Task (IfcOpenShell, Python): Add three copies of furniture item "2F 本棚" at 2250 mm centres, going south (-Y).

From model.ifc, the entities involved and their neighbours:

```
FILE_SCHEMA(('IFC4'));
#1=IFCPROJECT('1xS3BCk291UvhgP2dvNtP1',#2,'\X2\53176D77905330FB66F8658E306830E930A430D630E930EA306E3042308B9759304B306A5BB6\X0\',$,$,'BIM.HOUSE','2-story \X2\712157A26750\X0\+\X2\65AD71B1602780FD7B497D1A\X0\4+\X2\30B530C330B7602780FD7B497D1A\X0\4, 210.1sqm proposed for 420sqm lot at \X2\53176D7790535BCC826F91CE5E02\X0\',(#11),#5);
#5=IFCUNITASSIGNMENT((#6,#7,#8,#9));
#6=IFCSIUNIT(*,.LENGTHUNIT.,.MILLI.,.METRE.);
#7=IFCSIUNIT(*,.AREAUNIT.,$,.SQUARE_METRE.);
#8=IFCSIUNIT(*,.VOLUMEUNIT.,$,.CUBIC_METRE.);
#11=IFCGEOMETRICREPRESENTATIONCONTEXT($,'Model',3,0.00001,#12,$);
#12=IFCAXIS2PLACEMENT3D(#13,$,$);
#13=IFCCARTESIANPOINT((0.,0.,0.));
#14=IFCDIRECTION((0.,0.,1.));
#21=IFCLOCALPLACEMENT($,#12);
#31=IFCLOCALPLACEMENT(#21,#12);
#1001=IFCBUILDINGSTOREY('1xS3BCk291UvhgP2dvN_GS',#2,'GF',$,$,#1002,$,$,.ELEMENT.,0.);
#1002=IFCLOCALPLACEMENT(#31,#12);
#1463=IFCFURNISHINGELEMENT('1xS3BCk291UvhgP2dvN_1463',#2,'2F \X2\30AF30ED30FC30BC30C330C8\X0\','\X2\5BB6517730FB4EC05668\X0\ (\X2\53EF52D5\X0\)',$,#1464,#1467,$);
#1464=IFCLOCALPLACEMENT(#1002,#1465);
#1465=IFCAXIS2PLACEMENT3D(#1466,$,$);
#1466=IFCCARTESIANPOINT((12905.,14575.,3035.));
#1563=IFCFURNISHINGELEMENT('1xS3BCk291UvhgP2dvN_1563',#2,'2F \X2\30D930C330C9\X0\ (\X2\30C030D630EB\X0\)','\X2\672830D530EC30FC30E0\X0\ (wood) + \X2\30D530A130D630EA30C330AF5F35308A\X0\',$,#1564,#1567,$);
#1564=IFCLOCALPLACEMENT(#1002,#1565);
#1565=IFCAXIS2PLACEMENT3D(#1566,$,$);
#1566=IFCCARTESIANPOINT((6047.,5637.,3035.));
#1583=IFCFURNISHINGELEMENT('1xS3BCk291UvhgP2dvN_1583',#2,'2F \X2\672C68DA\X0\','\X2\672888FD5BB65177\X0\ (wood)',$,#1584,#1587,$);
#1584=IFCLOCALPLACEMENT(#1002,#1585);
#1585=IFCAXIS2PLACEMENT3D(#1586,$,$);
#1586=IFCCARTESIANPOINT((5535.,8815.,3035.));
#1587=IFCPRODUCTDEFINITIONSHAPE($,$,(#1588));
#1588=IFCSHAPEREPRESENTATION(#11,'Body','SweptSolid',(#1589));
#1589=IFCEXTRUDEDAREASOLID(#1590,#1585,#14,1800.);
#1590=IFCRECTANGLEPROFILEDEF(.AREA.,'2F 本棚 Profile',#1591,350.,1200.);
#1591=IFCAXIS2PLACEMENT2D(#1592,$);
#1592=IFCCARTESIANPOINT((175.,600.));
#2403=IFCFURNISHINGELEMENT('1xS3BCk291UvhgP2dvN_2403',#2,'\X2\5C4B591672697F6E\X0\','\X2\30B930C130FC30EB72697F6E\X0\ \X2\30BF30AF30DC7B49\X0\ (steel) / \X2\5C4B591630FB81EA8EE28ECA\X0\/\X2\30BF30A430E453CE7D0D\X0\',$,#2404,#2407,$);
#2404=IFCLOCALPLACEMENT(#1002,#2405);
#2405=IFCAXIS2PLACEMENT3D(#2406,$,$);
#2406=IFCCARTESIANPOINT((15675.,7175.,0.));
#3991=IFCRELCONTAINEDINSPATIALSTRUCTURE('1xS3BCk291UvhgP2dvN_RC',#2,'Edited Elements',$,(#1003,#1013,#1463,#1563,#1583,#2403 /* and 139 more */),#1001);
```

```python
import numpy as np
import ifcopenshell
import ifcopenshell.api.geometry
import ifcopenshell.api.root
import ifcopenshell.util.element
import ifcopenshell.util.placement
import ifcopenshell.util.unit

model = ifcopenshell.open("model.ifc")
unit_scale = ifcopenshell.util.unit.calculate_unit_scale(model)


def reuse_history(source, copy):
    """copy_class also copies each property set's owner history, people and application; keep the originals."""
    for rel in copy.IsDefinedBy:
        if rel.is_a("IfcRelDefinesByProperties") and (history := rel.RelatingPropertyDefinition.OwnerHistory):
            rel.RelatingPropertyDefinition.OwnerHistory = source.OwnerHistory
            ifcopenshell.util.element.remove_deep2(model, history)


source = model.by_guid("1xS3BCk291UvhgP2dvN_1583")
base = ifcopenshell.util.placement.get_local_placement(source.ObjectPlacement)
step = np.array([0.0, -1.0, 0.0]) * 2.25 / unit_scale

for i in range(1, 4):
    copy = ifcopenshell.api.root.copy_class(model, product=source)
    copy.Representation = ifcopenshell.util.element.copy_deep(
        model, source.Representation, exclude=["IfcGeometricRepresentationContext", "IfcRepresentationMap"]
    )
    reuse_history(source, copy)
    matrix = base.copy()
    matrix[:3, 3] += i * step
    print("added at", matrix[:3, 3].round(3) + 0.0)
    ifcopenshell.api.geometry.edit_object_placement(model, product=copy, matrix=matrix, is_si=False)

model.write("model_edited.ifc")
```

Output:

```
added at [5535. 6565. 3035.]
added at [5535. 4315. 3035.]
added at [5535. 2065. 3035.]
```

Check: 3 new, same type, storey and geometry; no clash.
